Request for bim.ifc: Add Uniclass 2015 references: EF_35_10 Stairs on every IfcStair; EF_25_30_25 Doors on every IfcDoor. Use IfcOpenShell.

First a look at what the model holds.

```python
import ifcopenshell

model = ifcopenshell.open("bim.ifc")
print(model.schema)
print("classifications:", [c.Name for c in model.by_type("IfcClassification")])
for ifc_class in ("IfcDoor", "IfcRoof", "IfcStair", "IfcWall", "IfcWindow"):
    print(ifc_class, len(model.by_type(ifc_class)))
```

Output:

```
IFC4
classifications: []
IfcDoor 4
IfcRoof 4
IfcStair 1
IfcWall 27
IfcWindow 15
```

```python
import ifcopenshell
import ifcopenshell.api.classification

model = ifcopenshell.open("bim.ifc")

system = ifcopenshell.api.classification.add_classification(model, classification="Uniclass 2015")

codes = {
    "IfcStair": ("EF_35_10", "Stairs"),
    "IfcDoor": ("EF_25_30_25", "Doors"),
}
for ifc_class, (code, name) in codes.items():
    products = model.by_type(ifc_class)
    ifcopenshell.api.classification.add_reference(
        model, products=products, classification=system, identification=code, name=name
    )
    print(code, len(products))

model.write("bim_rev.ifc")
```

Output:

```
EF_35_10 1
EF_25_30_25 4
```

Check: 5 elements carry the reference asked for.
